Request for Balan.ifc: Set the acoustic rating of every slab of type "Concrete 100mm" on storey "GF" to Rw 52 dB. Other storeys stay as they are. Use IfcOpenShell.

First a look at what the model holds.

```python
import ifcopenshell
import ifcopenshell.util.element

model = ifcopenshell.open("Balan.ifc")
print(model.schema)
storey = next(s for s in model.by_type("IfcBuildingStorey") if s.Name == "GF")
slabs = [e for e in ifcopenshell.util.element.get_decomposition(storey) if e.is_a("IfcSlab")]
seen = {}
for e in slabs:
    element_type = ifcopenshell.util.element.get_type(e)
    key = (element_type.Name if element_type != e and element_type else None, ifcopenshell.util.element.get_pset(e, "Pset_SlabCommon", "AcousticRating"))
    seen[key] = seen.get(key, 0) + 1
for (name, value), count in sorted(seen.items(), key=str):
    print(count, "x", name, "|", value)
```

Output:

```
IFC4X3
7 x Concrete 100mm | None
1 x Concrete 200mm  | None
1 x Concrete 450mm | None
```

```python
import ifcopenshell
import ifcopenshell.api.pset
import ifcopenshell.util.element

model = ifcopenshell.open("Balan.ifc")

storey = next(s for s in model.by_type("IfcBuildingStorey") if s.Name == "GF")
slabs = [e for e in ifcopenshell.util.element.get_decomposition(storey) if e.is_a("IfcSlab")]

count = 0
for e in slabs:
    element_type = ifcopenshell.util.element.get_type(e)
    if element_type in (None, e) or element_type.Name != "Concrete 100mm":
        continue
    # add_pset returns the element's existing set when there is one.
    pset = ifcopenshell.api.pset.add_pset(model, product=e, name="Pset_SlabCommon")
    ifcopenshell.api.pset.edit_pset(model, pset=pset, properties={"AcousticRating": "Rw 52 dB"})
    count += 1

print(count, "slabs updated")

model.write("Balan_edited.ifc")
```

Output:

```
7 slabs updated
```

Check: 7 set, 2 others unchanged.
